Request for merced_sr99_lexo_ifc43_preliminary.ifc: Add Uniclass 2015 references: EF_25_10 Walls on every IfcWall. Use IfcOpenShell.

First a look at what the model holds.

```python
import ifcopenshell

model = ifcopenshell.open("merced_sr99_lexo_ifc43_preliminary.ifc")
print(model.schema)
print("classifications:", [c.Name for c in model.by_type("IfcClassification")])
for ifc_class in ("IfcDoor", "IfcRoof", "IfcStair", "IfcWall", "IfcWindow"):
    print(ifc_class, len(model.by_type(ifc_class)))
```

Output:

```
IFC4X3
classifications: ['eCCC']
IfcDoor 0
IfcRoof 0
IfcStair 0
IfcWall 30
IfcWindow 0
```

```python
import ifcopenshell
import ifcopenshell.api.classification

model = ifcopenshell.open("merced_sr99_lexo_ifc43_preliminary.ifc")

system = ifcopenshell.api.classification.add_classification(model, classification="Uniclass 2015")

codes = {
    "IfcWall": ("EF_25_10", "Walls"),
}
for ifc_class, (code, name) in codes.items():
    products = model.by_type(ifc_class)
    ifcopenshell.api.classification.add_reference(
        model, products=products, classification=system, identification=code, name=name
    )
    print(code, len(products))

model.write("merced_sr99_lexo_ifc43_preliminary_updated.ifc")
```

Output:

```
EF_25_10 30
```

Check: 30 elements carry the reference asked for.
